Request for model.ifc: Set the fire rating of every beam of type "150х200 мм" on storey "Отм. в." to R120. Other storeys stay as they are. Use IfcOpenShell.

First a look at what the model holds.

```python
import ifcopenshell
import ifcopenshell.util.element

model = ifcopenshell.open("model.ifc")
print(model.schema)
storey = next(s for s in model.by_type("IfcBuildingStorey") if s.Name == "Отм. в.")
beams = [e for e in ifcopenshell.util.element.get_decomposition(storey) if e.is_a("IfcBeam")]
seen = {}
for e in beams:
    element_type = ifcopenshell.util.element.get_type(e)
    key = (element_type.Name if element_type != e and element_type else None, ifcopenshell.util.element.get_pset(e, "Pset_BeamCommon", "FireRating"))
    seen[key] = seen.get(key, 0) + 1
for (name, value), count in sorted(seen.items(), key=str):
    print(count, "x", name, "|", value)
```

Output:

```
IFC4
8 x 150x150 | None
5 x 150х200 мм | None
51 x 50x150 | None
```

```python
import ifcopenshell
import ifcopenshell.api.pset
import ifcopenshell.util.element

model = ifcopenshell.open("model.ifc")

storey = next(s for s in model.by_type("IfcBuildingStorey") if s.Name == "Отм. в.")
beams = [e for e in ifcopenshell.util.element.get_decomposition(storey) if e.is_a("IfcBeam")]

count = 0
for e in beams:
    element_type = ifcopenshell.util.element.get_type(e)
    if element_type in (None, e) or element_type.Name != "150х200 мм":
        continue
    # add_pset returns the element's existing set when there is one.
    pset = ifcopenshell.api.pset.add_pset(model, product=e, name="Pset_BeamCommon")
    ifcopenshell.api.pset.edit_pset(model, pset=pset, properties={"FireRating": "R120"})
    count += 1

print(count, "beams updated")

model.write("model_rev.ifc")
```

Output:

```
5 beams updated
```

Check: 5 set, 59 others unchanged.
